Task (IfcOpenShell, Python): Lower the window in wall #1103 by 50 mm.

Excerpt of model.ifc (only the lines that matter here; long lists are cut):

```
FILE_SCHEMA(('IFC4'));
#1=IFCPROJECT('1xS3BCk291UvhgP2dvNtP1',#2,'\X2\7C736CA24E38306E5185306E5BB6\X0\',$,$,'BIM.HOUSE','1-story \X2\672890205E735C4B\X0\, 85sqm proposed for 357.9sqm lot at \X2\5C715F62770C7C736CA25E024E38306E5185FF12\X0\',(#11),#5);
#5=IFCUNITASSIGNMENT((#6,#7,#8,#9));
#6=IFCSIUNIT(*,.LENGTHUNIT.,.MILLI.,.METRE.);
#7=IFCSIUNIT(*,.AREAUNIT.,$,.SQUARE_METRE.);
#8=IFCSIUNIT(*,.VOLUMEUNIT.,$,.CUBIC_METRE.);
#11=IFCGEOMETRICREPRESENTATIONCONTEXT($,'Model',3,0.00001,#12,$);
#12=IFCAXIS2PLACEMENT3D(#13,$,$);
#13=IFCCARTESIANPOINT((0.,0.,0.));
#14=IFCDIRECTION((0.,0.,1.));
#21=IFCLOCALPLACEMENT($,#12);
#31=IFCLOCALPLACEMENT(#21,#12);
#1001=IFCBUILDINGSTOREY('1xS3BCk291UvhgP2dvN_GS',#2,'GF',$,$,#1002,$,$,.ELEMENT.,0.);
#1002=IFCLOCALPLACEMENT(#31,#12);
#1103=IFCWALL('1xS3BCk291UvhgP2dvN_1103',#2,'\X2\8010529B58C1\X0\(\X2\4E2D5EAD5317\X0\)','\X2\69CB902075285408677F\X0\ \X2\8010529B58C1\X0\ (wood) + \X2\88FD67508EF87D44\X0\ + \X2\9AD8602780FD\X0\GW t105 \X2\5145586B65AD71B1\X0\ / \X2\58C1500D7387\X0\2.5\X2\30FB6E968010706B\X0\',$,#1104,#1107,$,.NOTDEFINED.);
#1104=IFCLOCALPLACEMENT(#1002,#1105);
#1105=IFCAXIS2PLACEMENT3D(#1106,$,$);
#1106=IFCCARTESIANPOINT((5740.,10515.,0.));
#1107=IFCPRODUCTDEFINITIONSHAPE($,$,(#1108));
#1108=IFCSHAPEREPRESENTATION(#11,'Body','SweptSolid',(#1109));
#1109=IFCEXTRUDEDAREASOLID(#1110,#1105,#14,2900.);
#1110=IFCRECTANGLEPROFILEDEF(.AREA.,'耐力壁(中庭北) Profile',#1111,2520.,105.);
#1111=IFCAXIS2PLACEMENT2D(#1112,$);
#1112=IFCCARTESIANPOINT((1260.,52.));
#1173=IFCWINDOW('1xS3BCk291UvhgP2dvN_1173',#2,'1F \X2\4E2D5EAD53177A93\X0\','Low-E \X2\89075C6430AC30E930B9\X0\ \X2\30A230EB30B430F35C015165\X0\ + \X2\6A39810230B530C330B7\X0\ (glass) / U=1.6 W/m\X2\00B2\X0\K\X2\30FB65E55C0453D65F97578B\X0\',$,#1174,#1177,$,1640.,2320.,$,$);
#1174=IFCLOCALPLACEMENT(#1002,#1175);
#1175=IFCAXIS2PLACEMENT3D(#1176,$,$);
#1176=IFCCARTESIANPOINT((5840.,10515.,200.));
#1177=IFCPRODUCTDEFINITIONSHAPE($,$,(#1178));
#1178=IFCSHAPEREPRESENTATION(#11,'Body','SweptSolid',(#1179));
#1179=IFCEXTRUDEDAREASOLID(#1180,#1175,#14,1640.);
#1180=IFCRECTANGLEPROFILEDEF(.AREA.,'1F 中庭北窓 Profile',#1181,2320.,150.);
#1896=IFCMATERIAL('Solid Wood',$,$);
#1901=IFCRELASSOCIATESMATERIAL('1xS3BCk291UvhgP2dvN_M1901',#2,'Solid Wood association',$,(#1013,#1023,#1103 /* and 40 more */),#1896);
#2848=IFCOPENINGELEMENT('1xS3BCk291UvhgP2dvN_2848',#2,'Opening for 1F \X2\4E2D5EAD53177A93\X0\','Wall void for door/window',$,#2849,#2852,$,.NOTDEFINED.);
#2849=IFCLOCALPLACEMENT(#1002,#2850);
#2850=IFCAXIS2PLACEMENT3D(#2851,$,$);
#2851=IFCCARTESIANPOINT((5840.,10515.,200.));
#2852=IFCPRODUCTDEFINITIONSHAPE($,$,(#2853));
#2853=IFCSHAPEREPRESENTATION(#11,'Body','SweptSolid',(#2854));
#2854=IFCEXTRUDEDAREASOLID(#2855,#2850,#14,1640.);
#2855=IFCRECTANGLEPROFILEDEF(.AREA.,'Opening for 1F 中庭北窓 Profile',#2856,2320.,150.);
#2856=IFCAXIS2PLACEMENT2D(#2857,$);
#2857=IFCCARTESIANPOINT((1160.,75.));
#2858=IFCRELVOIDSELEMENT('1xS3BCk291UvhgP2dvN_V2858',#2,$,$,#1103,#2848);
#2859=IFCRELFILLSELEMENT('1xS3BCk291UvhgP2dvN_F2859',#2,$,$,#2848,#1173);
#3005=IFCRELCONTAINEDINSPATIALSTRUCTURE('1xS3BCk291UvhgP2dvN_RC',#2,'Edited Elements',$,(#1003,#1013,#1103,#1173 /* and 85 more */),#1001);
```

```python
import numpy as np
import ifcopenshell
import ifcopenshell.api.geometry
import ifcopenshell.util.placement
import ifcopenshell.util.unit

model = ifcopenshell.open("model.ifc")
unit_scale = ifcopenshell.util.unit.calculate_unit_scale(model)

window = model.by_guid("1xS3BCk291UvhgP2dvN_1173")
opening = window.FillsVoids[0].RelatingOpeningElement
dz = -50.0

shift = np.array([0.0, 0.0, dz])
# The window is not placed relative to its opening, so move both.
for product in (opening, window):
    matrix = ifcopenshell.util.placement.get_local_placement(product.ObjectPlacement)
    matrix[:3, 3] += shift
    ifcopenshell.api.geometry.edit_object_placement(model, product=product, matrix=matrix, is_si=False)

print(f"moved by {dz * unit_scale:+.3f} m")

model.write("model-out.ifc")
```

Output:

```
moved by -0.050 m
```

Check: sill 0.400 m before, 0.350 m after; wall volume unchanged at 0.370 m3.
